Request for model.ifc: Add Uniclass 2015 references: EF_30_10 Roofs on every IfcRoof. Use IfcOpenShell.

First a look at what the model holds.

```python
import ifcopenshell

model = ifcopenshell.open("model.ifc")
print(model.schema)
print("classifications:", [c.Name for c in model.by_type("IfcClassification")])
for ifc_class in ("IfcDoor", "IfcRoof", "IfcStair", "IfcWall", "IfcWindow"):
    print(ifc_class, len(model.by_type(ifc_class)))
```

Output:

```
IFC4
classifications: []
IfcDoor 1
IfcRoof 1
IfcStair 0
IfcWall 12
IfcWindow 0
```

```python
import ifcopenshell
import ifcopenshell.api.classification

model = ifcopenshell.open("model.ifc")

system = ifcopenshell.api.classification.add_classification(model, classification="Uniclass 2015")

codes = {
    "IfcRoof": ("EF_30_10", "Roofs"),
}
for ifc_class, (code, name) in codes.items():
    products = model.by_type(ifc_class)
    ifcopenshell.api.classification.add_reference(
        model, products=products, classification=system, identification=code, name=name
    )
    print(code, len(products))

model.write("model_v2.ifc")
```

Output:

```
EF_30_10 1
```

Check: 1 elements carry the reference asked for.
